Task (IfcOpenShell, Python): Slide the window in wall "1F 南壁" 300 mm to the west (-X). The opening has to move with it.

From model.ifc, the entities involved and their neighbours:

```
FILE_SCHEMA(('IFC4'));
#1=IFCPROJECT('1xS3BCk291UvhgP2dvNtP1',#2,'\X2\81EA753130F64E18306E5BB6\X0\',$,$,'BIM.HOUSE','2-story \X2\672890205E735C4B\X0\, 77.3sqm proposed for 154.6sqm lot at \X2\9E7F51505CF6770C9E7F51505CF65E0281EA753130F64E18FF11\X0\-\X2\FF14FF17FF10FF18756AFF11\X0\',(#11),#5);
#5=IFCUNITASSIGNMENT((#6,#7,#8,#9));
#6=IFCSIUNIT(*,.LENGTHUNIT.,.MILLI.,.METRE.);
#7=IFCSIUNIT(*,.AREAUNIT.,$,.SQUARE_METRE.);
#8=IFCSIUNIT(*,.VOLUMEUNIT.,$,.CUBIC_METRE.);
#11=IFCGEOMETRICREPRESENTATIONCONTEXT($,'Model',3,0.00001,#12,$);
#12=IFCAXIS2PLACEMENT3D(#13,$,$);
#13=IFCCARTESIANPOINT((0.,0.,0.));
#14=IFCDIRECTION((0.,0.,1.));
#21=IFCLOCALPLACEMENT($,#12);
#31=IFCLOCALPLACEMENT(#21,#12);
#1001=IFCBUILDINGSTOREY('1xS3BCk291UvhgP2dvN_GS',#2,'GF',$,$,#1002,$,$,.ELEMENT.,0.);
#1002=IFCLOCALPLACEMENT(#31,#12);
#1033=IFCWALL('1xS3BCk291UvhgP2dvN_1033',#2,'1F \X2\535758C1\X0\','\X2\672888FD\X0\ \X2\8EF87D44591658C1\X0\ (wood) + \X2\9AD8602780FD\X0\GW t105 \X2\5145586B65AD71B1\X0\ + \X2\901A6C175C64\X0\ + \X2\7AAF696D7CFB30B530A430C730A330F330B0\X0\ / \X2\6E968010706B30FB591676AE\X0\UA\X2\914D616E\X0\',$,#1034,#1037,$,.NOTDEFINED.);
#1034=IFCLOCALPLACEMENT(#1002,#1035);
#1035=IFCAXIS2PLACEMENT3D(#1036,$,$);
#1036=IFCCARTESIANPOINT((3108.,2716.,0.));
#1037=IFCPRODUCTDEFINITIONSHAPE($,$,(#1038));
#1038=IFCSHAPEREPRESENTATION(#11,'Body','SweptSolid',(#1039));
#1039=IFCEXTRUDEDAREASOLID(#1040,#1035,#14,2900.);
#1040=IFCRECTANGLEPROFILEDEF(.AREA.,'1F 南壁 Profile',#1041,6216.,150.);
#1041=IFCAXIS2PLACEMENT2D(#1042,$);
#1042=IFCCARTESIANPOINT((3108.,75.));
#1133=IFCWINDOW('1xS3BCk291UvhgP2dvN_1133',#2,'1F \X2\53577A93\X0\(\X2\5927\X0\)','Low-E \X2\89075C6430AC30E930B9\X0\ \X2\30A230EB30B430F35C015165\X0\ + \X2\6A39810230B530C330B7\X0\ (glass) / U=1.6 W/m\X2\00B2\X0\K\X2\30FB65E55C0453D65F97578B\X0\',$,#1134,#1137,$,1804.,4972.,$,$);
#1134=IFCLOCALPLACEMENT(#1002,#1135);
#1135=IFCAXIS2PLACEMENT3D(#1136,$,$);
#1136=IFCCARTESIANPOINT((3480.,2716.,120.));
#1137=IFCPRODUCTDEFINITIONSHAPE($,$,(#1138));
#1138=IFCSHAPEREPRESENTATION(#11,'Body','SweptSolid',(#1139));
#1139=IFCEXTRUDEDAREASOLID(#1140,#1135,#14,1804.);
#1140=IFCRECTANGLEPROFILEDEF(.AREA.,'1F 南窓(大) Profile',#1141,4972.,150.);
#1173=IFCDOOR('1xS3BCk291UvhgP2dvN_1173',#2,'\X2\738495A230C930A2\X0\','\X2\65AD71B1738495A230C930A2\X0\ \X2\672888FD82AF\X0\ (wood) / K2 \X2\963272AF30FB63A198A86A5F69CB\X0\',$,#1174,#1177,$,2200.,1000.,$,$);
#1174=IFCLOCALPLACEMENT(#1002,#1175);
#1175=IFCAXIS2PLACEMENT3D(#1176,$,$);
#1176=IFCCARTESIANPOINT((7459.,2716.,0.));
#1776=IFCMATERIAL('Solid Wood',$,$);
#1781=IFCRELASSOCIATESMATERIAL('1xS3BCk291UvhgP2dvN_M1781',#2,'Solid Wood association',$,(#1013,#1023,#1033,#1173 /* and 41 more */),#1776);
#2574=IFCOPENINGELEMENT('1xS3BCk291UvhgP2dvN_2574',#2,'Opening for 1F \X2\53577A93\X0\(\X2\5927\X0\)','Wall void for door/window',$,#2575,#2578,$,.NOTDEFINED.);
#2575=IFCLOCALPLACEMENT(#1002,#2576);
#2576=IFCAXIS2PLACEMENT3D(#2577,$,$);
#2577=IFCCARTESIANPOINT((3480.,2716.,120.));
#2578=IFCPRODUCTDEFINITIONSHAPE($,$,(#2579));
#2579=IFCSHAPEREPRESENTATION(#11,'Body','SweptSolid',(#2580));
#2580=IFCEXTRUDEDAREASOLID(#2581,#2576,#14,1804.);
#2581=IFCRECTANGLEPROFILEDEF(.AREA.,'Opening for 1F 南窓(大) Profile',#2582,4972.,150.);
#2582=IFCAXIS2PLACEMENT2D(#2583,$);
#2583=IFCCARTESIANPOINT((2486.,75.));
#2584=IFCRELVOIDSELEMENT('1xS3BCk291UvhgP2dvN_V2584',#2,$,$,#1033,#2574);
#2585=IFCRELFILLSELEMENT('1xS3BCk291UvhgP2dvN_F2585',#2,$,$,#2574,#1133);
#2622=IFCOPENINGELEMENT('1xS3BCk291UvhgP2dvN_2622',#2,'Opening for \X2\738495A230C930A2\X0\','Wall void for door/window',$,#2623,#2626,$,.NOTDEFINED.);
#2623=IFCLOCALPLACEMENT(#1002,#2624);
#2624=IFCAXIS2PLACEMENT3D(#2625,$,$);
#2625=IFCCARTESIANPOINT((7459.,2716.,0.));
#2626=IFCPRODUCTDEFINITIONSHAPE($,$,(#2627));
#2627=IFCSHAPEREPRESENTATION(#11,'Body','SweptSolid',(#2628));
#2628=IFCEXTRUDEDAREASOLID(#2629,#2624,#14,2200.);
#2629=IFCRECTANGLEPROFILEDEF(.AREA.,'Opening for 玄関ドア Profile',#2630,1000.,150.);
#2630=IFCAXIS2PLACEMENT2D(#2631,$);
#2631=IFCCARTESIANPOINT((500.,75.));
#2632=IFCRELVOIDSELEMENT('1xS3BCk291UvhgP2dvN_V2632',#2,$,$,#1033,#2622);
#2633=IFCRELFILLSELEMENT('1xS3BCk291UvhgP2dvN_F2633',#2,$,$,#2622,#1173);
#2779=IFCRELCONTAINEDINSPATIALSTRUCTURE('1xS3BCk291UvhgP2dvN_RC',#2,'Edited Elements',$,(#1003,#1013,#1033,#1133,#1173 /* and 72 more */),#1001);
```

```python
import ifcopenshell
import ifcopenshell.api.geometry
import ifcopenshell.util.placement
import ifcopenshell.util.unit

model = ifcopenshell.open("model.ifc")
unit_scale = ifcopenshell.util.unit.calculate_unit_scale(model)

window = model.by_guid("1xS3BCk291UvhgP2dvN_1133")
opening = window.FillsVoids[0].RelatingOpeningElement
wall = opening.VoidsElements[0].RelatingBuildingElement

wall_matrix = ifcopenshell.util.placement.get_local_placement(wall.ObjectPlacement)
shift = wall_matrix[:3, 0] * -0.3 / unit_scale
before = ifcopenshell.util.placement.get_local_placement(window.ObjectPlacement)[:3, 3].copy()

# The window is not placed relative to its opening, so move both.
for product in (opening, window):
    matrix = ifcopenshell.util.placement.get_local_placement(product.ObjectPlacement)
    matrix[:3, 3] += shift
    ifcopenshell.api.geometry.edit_object_placement(model, product=product, matrix=matrix, is_si=False)

after = ifcopenshell.util.placement.get_local_placement(window.ObjectPlacement)[:3, 3]
print("window moved by", (after - before).round(3) + 0.0)

model.write("model_v2.ifc")
```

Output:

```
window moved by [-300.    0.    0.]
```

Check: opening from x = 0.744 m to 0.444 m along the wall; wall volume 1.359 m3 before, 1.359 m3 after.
